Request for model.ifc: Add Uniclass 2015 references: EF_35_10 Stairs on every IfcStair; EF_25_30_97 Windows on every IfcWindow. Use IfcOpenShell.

First a look at what the model holds.

```python
import ifcopenshell

model = ifcopenshell.open("model.ifc")
print(model.schema)
print("classifications:", [c.Name for c in model.by_type("IfcClassification")])
for ifc_class in ("IfcDoor", "IfcRoof", "IfcStair", "IfcWall", "IfcWindow"):
    print(ifc_class, len(model.by_type(ifc_class)))
```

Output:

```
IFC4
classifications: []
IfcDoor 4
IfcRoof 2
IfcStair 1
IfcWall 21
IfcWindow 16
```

```python
import ifcopenshell
import ifcopenshell.api.classification

model = ifcopenshell.open("model.ifc")

system = ifcopenshell.api.classification.add_classification(model, classification="Uniclass 2015")

codes = {
    "IfcStair": ("EF_35_10", "Stairs"),
    "IfcWindow": ("EF_25_30_97", "Windows"),
}
for ifc_class, (code, name) in codes.items():
    products = model.by_type(ifc_class)
    ifcopenshell.api.classification.add_reference(
        model, products=products, classification=system, identification=code, name=name
    )
    print(code, len(products))

model.write("model_v2.ifc")
```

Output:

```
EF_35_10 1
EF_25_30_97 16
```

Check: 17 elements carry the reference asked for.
